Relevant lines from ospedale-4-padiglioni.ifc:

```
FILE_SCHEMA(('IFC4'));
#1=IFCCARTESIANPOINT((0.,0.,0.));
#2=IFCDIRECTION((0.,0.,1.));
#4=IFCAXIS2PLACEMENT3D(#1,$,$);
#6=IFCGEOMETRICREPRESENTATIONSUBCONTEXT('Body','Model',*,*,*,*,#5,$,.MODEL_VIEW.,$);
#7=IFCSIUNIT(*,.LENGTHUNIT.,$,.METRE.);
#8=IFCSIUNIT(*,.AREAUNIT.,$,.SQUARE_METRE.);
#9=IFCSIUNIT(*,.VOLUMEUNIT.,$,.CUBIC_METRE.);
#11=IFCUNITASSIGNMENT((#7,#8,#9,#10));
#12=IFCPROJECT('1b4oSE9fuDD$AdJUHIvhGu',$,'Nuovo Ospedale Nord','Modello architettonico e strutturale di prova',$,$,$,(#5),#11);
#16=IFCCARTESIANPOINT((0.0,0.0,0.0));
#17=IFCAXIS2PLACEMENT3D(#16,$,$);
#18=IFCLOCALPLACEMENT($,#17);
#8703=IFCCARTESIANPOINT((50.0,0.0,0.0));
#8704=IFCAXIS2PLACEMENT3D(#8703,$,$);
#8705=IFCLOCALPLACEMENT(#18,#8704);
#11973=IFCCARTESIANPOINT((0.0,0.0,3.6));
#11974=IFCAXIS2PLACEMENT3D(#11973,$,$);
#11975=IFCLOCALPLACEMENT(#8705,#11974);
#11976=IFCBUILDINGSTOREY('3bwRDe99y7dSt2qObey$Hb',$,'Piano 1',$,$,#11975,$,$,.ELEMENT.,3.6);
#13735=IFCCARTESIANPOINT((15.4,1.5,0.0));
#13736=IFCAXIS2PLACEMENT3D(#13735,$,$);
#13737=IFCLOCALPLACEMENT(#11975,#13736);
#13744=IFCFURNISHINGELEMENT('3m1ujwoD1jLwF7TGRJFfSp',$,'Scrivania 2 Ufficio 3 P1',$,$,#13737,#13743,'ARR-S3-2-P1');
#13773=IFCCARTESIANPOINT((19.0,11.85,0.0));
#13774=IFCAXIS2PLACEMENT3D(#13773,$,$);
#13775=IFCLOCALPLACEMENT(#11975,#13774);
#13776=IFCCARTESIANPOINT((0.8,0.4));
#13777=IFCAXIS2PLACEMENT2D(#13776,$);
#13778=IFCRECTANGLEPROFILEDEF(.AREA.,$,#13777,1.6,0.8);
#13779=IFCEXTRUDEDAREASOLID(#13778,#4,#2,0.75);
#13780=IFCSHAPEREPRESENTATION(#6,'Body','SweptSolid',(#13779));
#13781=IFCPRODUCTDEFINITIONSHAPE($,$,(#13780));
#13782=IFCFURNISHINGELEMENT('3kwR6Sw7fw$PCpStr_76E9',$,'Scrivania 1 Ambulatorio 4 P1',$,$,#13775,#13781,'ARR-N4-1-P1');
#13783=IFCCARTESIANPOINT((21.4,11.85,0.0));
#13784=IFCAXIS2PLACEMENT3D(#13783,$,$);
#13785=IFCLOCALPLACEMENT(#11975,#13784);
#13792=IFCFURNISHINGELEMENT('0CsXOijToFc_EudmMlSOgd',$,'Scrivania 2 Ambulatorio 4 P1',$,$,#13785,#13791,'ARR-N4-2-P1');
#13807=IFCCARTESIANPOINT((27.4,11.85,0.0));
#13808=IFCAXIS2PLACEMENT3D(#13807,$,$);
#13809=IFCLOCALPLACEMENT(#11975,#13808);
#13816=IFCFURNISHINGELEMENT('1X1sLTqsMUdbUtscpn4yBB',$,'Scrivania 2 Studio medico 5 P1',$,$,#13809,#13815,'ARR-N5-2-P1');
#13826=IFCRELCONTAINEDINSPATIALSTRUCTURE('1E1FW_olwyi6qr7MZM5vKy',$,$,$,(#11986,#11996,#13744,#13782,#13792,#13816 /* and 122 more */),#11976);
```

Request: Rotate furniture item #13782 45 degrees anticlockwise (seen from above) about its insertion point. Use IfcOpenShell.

```python
import ifcopenshell
import ifcopenshell.api.geometry
import ifcopenshell.util.placement

model = ifcopenshell.open("ospedale-4-padiglioni.ifc")

item = model.by_id(13782)
matrix = ifcopenshell.util.placement.get_local_placement(item.ObjectPlacement)
matrix = matrix @ ifcopenshell.util.placement.rotation(45, "Z")
ifcopenshell.api.geometry.edit_object_placement(model, product=item, matrix=matrix, is_si=False)

print(ifcopenshell.util.placement.get_local_placement(item.ObjectPlacement).round(3) + 0.0)

model.write("ospedale-4-padiglioni_rev.ifc")
```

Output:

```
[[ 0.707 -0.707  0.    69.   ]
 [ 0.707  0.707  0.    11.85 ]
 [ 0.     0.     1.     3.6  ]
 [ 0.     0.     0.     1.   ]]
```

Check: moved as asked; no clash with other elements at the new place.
